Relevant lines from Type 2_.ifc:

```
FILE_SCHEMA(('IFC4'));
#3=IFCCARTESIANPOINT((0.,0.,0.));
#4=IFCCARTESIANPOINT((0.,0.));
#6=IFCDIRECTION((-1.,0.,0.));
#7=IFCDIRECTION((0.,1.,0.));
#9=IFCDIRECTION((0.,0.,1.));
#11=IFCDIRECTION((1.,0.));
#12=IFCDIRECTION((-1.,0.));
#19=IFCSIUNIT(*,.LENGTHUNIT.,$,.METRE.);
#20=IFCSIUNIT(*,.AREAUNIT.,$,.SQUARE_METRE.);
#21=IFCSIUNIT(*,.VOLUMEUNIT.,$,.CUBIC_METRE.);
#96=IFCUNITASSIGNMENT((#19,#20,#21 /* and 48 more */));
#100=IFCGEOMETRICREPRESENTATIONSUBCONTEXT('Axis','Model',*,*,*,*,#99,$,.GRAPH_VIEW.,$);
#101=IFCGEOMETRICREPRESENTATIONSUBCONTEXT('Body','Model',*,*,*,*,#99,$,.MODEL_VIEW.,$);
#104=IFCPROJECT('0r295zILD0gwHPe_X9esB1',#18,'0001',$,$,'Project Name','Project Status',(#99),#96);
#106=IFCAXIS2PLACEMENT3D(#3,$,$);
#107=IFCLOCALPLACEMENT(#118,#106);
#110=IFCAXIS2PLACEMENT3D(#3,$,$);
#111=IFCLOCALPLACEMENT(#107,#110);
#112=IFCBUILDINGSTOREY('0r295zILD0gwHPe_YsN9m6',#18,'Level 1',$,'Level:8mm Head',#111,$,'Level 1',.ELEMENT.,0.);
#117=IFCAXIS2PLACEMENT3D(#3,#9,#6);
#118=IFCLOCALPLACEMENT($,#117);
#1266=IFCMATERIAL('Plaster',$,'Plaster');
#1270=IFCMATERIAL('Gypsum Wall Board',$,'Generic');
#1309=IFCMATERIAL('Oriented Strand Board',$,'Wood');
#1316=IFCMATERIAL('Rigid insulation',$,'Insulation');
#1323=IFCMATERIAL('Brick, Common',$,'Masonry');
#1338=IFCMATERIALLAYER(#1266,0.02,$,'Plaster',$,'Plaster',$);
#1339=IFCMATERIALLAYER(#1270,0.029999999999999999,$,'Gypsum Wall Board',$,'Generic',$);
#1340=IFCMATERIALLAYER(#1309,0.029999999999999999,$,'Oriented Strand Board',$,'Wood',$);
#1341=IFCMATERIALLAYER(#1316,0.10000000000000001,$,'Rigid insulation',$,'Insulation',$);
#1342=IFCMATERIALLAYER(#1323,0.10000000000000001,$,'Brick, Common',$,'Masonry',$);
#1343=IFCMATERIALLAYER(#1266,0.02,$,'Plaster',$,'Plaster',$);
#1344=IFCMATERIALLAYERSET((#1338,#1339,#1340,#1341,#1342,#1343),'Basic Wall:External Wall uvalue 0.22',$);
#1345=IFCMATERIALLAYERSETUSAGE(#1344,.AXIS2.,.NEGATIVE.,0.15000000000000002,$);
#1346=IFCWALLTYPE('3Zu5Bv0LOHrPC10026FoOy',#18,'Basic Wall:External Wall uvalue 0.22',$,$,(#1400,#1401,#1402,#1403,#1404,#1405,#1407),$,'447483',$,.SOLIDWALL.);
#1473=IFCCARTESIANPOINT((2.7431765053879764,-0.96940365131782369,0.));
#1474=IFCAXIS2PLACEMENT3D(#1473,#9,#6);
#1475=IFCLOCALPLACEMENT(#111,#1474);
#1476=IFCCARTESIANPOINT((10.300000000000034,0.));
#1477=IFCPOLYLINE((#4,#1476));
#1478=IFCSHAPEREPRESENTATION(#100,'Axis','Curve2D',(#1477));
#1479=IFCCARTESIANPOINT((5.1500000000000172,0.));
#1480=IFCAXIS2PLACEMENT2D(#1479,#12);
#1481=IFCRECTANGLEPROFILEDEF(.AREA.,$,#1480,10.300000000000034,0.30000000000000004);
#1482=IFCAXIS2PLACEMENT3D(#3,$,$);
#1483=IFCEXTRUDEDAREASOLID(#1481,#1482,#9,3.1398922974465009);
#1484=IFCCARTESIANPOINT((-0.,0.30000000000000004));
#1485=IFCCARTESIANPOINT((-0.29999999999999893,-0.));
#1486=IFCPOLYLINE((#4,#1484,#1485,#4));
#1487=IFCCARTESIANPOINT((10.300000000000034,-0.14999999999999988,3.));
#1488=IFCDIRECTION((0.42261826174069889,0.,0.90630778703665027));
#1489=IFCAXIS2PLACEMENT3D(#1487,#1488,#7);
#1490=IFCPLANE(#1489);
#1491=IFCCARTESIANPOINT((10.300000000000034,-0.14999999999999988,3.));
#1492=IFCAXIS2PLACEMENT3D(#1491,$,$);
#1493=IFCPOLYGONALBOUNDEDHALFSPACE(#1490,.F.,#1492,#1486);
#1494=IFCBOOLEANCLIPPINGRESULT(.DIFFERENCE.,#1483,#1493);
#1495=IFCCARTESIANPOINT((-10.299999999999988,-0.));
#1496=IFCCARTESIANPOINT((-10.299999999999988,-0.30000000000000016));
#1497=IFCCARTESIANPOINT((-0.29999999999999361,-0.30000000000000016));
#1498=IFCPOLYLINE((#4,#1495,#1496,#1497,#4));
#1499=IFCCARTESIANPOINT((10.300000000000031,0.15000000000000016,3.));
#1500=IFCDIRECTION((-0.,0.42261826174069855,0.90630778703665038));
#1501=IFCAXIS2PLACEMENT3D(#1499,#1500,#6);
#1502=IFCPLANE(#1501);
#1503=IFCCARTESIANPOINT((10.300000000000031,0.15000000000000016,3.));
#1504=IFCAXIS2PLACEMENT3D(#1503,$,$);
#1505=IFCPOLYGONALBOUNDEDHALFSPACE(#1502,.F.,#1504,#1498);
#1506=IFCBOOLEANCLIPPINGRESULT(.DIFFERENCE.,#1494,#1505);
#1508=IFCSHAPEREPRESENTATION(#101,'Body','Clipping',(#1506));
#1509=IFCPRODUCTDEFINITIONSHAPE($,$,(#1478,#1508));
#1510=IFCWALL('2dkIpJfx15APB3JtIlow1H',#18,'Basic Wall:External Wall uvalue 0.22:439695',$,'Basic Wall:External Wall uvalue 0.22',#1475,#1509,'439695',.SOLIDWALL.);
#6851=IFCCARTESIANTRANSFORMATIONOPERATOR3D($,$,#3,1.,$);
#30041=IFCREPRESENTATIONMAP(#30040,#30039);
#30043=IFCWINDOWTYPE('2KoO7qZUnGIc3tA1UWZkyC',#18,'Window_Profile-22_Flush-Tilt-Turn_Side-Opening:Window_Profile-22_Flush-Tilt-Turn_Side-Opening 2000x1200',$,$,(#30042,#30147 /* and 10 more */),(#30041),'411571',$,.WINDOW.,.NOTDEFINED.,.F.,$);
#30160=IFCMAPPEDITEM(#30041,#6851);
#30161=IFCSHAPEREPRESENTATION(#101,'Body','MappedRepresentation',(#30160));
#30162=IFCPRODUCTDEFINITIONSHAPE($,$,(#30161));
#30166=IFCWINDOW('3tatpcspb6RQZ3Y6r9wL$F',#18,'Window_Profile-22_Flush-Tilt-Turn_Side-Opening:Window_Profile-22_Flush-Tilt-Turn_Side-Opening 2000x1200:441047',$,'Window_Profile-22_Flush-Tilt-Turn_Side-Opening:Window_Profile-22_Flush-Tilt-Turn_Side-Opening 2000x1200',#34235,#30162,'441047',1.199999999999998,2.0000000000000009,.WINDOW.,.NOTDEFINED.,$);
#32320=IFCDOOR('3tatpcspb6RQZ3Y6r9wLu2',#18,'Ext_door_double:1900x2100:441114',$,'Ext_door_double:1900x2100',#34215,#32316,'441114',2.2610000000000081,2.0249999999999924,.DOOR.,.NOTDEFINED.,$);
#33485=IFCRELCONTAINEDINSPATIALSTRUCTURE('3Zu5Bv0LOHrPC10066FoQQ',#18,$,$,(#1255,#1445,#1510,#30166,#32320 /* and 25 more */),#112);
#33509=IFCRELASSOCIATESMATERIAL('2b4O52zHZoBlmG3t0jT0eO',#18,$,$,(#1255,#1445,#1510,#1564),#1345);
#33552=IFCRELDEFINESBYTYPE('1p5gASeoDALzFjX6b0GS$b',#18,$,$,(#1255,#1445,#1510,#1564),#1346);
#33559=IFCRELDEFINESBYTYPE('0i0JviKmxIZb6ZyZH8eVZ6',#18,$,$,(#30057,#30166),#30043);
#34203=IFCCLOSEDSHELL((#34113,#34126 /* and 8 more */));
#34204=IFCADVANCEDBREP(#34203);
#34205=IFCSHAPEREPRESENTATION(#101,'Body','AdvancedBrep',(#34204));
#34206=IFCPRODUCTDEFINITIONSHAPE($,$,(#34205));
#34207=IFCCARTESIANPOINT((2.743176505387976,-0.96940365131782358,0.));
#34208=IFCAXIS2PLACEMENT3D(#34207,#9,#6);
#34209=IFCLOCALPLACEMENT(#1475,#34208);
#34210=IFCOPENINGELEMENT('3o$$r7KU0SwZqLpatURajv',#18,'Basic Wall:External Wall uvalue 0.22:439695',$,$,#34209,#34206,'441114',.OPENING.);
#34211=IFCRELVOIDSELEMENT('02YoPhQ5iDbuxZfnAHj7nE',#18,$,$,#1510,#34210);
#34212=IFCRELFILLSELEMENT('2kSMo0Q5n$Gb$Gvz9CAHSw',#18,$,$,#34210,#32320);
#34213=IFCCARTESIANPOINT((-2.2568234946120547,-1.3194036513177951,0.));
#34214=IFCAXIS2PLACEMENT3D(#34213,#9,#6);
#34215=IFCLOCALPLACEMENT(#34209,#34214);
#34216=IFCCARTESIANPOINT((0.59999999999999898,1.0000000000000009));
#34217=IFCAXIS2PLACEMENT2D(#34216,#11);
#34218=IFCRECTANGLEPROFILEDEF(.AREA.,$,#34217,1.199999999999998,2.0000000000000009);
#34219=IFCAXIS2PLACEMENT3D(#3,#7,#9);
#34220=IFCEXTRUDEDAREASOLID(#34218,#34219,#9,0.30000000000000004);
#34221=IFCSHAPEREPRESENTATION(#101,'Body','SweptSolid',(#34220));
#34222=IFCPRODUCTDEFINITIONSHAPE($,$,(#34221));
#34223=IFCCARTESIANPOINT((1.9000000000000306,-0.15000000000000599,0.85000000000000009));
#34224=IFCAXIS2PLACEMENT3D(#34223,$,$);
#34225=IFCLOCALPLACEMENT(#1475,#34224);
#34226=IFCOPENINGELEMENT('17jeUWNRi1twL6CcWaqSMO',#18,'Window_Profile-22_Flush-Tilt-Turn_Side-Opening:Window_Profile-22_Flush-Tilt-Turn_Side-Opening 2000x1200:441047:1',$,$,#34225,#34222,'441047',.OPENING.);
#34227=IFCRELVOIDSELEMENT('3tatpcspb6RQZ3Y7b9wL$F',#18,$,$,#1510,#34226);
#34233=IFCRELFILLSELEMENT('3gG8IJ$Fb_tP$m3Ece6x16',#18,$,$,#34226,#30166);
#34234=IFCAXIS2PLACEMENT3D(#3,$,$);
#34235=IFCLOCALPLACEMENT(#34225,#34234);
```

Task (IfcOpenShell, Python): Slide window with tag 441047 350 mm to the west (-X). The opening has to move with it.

```python
import ifcopenshell
import ifcopenshell.api.geometry
import ifcopenshell.util.placement
import ifcopenshell.util.unit

model = ifcopenshell.open("Type 2_.ifc")
unit_scale = ifcopenshell.util.unit.calculate_unit_scale(model)

window = model.by_guid("3tatpcspb6RQZ3Y6r9wL$F")
opening = window.FillsVoids[0].RelatingOpeningElement
wall = opening.VoidsElements[0].RelatingBuildingElement

wall_matrix = ifcopenshell.util.placement.get_local_placement(wall.ObjectPlacement)
shift = wall_matrix[:3, 0] * -0.35 / unit_scale
before = ifcopenshell.util.placement.get_local_placement(window.ObjectPlacement)[:3, 3].copy()

# The window is placed relative to its opening, so it follows when the opening moves.
matrix = ifcopenshell.util.placement.get_local_placement(opening.ObjectPlacement)
matrix[:3, 3] += shift
ifcopenshell.api.geometry.edit_object_placement(
    model, product=opening, matrix=matrix, is_si=False, should_transform_children=True
)

after = ifcopenshell.util.placement.get_local_placement(window.ObjectPlacement)[:3, 3]
print("window moved by", (after - before).round(3) + 0.0)

model.write("Type 2_-out.ifc")
```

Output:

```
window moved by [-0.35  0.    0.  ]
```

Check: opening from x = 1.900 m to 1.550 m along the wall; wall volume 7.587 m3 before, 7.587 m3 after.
